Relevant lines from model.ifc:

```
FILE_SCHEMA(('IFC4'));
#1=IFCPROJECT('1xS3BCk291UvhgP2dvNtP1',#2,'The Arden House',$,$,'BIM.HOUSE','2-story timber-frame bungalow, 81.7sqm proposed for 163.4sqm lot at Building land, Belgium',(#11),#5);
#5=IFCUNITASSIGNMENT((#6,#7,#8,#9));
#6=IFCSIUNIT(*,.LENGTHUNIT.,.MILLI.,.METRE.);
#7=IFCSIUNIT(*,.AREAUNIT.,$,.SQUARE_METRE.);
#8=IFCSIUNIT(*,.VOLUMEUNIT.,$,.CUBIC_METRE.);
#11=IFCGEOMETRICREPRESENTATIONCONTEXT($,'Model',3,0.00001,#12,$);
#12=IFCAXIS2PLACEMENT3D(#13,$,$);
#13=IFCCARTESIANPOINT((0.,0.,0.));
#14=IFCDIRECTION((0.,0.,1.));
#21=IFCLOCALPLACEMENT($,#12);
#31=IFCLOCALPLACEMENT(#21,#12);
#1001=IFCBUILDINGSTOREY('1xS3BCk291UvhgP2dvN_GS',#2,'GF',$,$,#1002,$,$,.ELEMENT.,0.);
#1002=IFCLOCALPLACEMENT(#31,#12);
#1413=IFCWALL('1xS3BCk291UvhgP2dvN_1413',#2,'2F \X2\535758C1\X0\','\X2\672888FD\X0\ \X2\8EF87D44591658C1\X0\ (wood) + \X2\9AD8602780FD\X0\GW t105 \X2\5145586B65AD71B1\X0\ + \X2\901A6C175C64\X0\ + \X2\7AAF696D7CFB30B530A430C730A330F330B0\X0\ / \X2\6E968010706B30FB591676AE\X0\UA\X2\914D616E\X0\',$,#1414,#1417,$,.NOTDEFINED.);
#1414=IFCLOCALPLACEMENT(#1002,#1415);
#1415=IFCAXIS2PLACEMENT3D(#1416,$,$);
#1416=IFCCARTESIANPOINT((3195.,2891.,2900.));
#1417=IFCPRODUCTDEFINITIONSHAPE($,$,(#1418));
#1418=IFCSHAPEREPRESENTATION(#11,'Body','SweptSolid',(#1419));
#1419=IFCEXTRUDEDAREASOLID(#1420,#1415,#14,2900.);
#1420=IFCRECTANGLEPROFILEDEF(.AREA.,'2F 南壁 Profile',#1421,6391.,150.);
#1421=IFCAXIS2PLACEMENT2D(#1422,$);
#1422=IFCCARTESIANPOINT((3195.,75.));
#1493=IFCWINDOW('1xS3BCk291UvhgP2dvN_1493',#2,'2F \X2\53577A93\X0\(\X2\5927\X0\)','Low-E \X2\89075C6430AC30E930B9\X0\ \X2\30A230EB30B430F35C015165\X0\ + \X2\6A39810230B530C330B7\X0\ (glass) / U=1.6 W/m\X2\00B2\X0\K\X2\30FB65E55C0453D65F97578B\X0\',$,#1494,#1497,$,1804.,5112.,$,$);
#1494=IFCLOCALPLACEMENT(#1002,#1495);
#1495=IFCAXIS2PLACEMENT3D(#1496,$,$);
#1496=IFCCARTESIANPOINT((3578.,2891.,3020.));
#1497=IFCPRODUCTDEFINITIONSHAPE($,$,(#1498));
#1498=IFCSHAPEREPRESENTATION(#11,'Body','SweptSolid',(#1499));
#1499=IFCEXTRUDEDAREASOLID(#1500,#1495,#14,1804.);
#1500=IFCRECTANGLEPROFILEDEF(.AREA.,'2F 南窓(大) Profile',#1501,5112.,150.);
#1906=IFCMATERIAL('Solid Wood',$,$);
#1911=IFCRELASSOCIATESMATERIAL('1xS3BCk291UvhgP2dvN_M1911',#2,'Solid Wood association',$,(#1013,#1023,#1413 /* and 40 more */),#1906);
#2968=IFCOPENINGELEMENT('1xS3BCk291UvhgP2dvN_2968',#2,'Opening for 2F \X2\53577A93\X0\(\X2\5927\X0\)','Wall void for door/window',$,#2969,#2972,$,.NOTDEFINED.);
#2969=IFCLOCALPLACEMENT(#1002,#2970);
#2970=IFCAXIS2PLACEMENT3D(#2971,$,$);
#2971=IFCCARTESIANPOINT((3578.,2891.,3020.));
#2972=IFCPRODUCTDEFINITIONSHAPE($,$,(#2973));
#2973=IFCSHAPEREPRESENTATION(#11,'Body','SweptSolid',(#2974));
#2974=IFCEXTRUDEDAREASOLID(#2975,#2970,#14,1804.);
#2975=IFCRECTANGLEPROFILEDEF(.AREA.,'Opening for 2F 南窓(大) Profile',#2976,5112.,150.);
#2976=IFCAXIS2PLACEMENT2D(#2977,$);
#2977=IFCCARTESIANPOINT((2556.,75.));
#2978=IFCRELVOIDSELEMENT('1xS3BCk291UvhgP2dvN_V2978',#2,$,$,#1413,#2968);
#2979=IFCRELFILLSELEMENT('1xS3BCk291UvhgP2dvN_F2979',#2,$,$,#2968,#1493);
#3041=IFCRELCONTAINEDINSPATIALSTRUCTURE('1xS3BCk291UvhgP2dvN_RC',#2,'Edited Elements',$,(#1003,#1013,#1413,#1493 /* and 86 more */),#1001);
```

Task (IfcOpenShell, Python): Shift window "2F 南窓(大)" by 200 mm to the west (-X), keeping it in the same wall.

```python
import ifcopenshell
import ifcopenshell.api.geometry
import ifcopenshell.util.placement

model = ifcopenshell.open("model.ifc")

window = model.by_id(1493)
opening = window.FillsVoids[0].RelatingOpeningElement
wall = opening.VoidsElements[0].RelatingBuildingElement

wall_matrix = ifcopenshell.util.placement.get_local_placement(wall.ObjectPlacement)
shift = wall_matrix[:3, 0] * -200.0
before = ifcopenshell.util.placement.get_local_placement(window.ObjectPlacement)[:3, 3].copy()

# The window is not placed relative to its opening, so move both.
for product in (opening, window):
    matrix = ifcopenshell.util.placement.get_local_placement(product.ObjectPlacement)
    matrix[:3, 3] += shift
    ifcopenshell.api.geometry.edit_object_placement(model, product=product, matrix=matrix, is_si=False)

after = ifcopenshell.util.placement.get_local_placement(window.ObjectPlacement)[:3, 3]
print("window moved by", (after - before).round(3) + 0.0)

model.write("model-out.ifc")
```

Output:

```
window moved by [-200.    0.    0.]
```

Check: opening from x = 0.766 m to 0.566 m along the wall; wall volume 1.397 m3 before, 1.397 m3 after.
